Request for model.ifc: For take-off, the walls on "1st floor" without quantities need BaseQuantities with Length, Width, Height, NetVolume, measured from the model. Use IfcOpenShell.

First a look at what the model holds.

```python
import ifcopenshell
import ifcopenshell.util.element
import ifcopenshell.util.unit

model = ifcopenshell.open("model.ifc")
print(model.schema)
for unit_type in ("LENGTHUNIT", "AREAUNIT", "VOLUMEUNIT"):
    print(unit_type, ifcopenshell.util.unit.calculate_unit_scale(model, unit_type))
storey = next(s for s in model.by_type("IfcBuildingStorey") if s.Name == "1st floor")
walls = [e for e in ifcopenshell.util.element.get_decomposition(storey) if e.is_a("IfcWall")]
for e in sorted(walls, key=lambda e: e.id()):
    print(e.id(), e.is_a(), e.Name, list(ifcopenshell.util.element.get_psets(e, qtos_only=True)), sep=" | ")
```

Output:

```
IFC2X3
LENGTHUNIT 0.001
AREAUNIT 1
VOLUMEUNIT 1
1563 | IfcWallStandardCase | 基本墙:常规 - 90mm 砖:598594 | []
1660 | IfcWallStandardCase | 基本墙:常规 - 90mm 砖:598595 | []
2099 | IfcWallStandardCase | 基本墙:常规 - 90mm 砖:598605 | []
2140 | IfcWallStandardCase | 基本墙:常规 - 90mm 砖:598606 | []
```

```python
import ifcopenshell
import ifcopenshell.api.pset
import ifcopenshell.geom
import ifcopenshell.util.element
import ifcopenshell.util.shape
import ifcopenshell.util.unit

model = ifcopenshell.open("model.ifc")
unit_scale = ifcopenshell.util.unit.calculate_unit_scale(model)
volume_scale = ifcopenshell.util.unit.calculate_unit_scale(model, "VOLUMEUNIT")
settings = ifcopenshell.geom.settings()

storey = next(s for s in model.by_type("IfcBuildingStorey") if s.Name == "1st floor")
walls = [e for e in ifcopenshell.util.element.get_decomposition(storey) if e.is_a("IfcWall")]

for e in sorted(walls, key=lambda e: e.id()):
    if ifcopenshell.util.element.get_psets(e, qtos_only=True, should_inherit=False):
        continue
    # Geometry comes back in metres, in the element's own axes.
    shape = ifcopenshell.geom.create_shape(settings, e)
    values = {
        "Length": ifcopenshell.util.shape.get_x(shape.geometry) / unit_scale,
        "Width": ifcopenshell.util.shape.get_y(shape.geometry) / unit_scale,
        "Height": ifcopenshell.util.shape.get_z(shape.geometry) / unit_scale,
        "NetVolume": ifcopenshell.util.shape.get_volume(shape.geometry) / volume_scale,
    }
    qto = ifcopenshell.api.pset.add_qto(model, product=e, name="BaseQuantities")
    ifcopenshell.api.pset.edit_qto(model, qto=qto, properties=values)
    print(e.id(), {k: round(v, 3) for k, v in values.items()})

model.write("model_v2.ifc")
```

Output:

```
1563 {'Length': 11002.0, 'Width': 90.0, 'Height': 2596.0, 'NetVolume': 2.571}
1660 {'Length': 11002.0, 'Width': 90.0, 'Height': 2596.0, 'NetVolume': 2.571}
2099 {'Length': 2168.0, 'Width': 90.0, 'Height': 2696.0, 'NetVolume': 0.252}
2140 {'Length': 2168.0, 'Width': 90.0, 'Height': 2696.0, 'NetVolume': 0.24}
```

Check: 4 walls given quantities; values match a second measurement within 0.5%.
